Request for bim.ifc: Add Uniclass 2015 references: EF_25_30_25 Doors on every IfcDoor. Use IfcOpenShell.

First a look at what the model holds.

```python
import ifcopenshell

model = ifcopenshell.open("bim.ifc")
print(model.schema)
print("classifications:", [c.Name for c in model.by_type("IfcClassification")])
for ifc_class in ("IfcDoor", "IfcRoof", "IfcStair", "IfcWall", "IfcWindow"):
    print(ifc_class, len(model.by_type(ifc_class)))
```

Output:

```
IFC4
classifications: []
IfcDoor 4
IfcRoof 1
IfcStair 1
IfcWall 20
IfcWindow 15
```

```python
import ifcopenshell
import ifcopenshell.api.classification

model = ifcopenshell.open("bim.ifc")

system = ifcopenshell.api.classification.add_classification(model, classification="Uniclass 2015")

codes = {
    "IfcDoor": ("EF_25_30_25", "Doors"),
}
for ifc_class, (code, name) in codes.items():
    products = model.by_type(ifc_class)
    ifcopenshell.api.classification.add_reference(
        model, products=products, classification=system, identification=code, name=name
    )
    print(code, len(products))

model.write("bim_v2.ifc")
```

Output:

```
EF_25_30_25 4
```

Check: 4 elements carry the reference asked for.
